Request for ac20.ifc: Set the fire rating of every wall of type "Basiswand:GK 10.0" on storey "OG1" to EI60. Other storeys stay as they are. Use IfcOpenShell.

First a look at what the model holds.

```python
import ifcopenshell
import ifcopenshell.util.element

model = ifcopenshell.open("ac20.ifc")
print(model.schema)
storey = next(s for s in model.by_type("IfcBuildingStorey") if s.Name == "OG1")
walls = [e for e in ifcopenshell.util.element.get_decomposition(storey) if e.is_a("IfcWall")]
seen = {}
for e in walls:
    element_type = ifcopenshell.util.element.get_type(e)
    key = (element_type.Name if element_type != e and element_type else None, ifcopenshell.util.element.get_pset(e, "Pset_WallCommon", "FireRating"))
    seen[key] = seen.get(key, 0) + 1
for (name, value), count in sorted(seen.items(), key=str):
    print(count, "x", name, "|", value)
```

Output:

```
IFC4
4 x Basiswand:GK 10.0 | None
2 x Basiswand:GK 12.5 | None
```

```python
import ifcopenshell
import ifcopenshell.api.pset
import ifcopenshell.util.element

model = ifcopenshell.open("ac20.ifc")

storey = next(s for s in model.by_type("IfcBuildingStorey") if s.Name == "OG1")
walls = [e for e in ifcopenshell.util.element.get_decomposition(storey) if e.is_a("IfcWall")]

count = 0
for e in walls:
    element_type = ifcopenshell.util.element.get_type(e)
    if element_type in (None, e) or element_type.Name != "Basiswand:GK 10.0":
        continue
    # add_pset returns the element's existing set when there is one.
    pset = ifcopenshell.api.pset.add_pset(model, product=e, name="Pset_WallCommon")
    ifcopenshell.api.pset.edit_pset(model, pset=pset, properties={"FireRating": "EI60"})
    count += 1

print(count, "walls updated")

model.write("ac20_rev.ifc")
```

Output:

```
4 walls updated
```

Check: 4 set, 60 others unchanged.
